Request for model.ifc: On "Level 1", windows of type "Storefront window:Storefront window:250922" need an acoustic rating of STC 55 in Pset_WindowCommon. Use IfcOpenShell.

First a look at what the model holds.

```python
import ifcopenshell
import ifcopenshell.util.element

model = ifcopenshell.open("model.ifc")
print(model.schema)
storey = next(s for s in model.by_type("IfcBuildingStorey") if s.Name == "Level 1")
windows = [e for e in ifcopenshell.util.element.get_decomposition(storey) if e.is_a("IfcWindow")]
seen = {}
for e in windows:
    element_type = ifcopenshell.util.element.get_type(e)
    key = (element_type.Name if element_type != e and element_type else None, ifcopenshell.util.element.get_pset(e, "Pset_WindowCommon", "AcousticRating"))
    seen[key] = seen.get(key, 0) + 1
for (name, value), count in sorted(seen.items(), key=str):
    print(count, "x", name, "|", value)
```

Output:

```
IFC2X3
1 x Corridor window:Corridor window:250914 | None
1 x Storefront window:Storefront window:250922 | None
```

```python
import ifcopenshell
import ifcopenshell.api.pset
import ifcopenshell.util.element

model = ifcopenshell.open("model.ifc")

storey = next(s for s in model.by_type("IfcBuildingStorey") if s.Name == "Level 1")
windows = [e for e in ifcopenshell.util.element.get_decomposition(storey) if e.is_a("IfcWindow")]

count = 0
for e in windows:
    element_type = ifcopenshell.util.element.get_type(e)
    if element_type in (None, e) or element_type.Name != "Storefront window:Storefront window:250922":
        continue
    # add_pset returns the element's existing set when there is one.
    pset = ifcopenshell.api.pset.add_pset(model, product=e, name="Pset_WindowCommon")
    ifcopenshell.api.pset.edit_pset(model, pset=pset, properties={"AcousticRating": "STC 55"})
    count += 1

print(count, "windows updated")

model.write("model_v2.ifc")
```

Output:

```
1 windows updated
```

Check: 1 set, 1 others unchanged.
